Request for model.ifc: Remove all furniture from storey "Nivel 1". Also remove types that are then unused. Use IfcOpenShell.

First a look at what the model holds.

```python
import ifcopenshell
import ifcopenshell.util.element

model = ifcopenshell.open("model.ifc")
print(model.schema)
storey = next(s for s in model.by_type("IfcBuildingStorey") if s.Name == "Nivel 1")
furniture = [e for e in ifcopenshell.util.element.get_decomposition(storey) if e.is_a("IfcFurnishingElement")]
seen = {}
for e in furniture:
    element_type = ifcopenshell.util.element.get_type(e)
    name = element_type.Name if element_type not in (None, e) else None
    seen[name] = seen.get(name, 0) + 1
for name, count in sorted(seen.items(), key=str):
    print(count, "x", name)
```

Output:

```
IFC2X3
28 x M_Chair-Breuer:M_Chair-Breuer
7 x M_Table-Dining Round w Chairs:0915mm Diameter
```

```python
import ifcopenshell
import ifcopenshell.api.root
import ifcopenshell.util.element

model = ifcopenshell.open("model.ifc")

storey = next(s for s in model.by_type("IfcBuildingStorey") if s.Name == "Nivel 1")
furniture = [e for e in ifcopenshell.util.element.get_decomposition(storey) if e.is_a("IfcFurnishingElement")]
types = {ifcopenshell.util.element.get_type(e) for e in furniture} - {None, *furniture}

for e in furniture:
    ifcopenshell.api.root.remove_product(model, product=e)
print(len(furniture), "removed")

unused = [t for t in types if not ifcopenshell.util.element.get_types(t)]
for t in unused:
    ifcopenshell.api.root.remove_product(model, product=t)
print(len(unused), "unused types removed")

model.write("model_v2.ifc")
```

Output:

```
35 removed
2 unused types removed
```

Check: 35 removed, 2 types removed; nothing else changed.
